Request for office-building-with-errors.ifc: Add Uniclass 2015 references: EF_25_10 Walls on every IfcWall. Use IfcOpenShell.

First a look at what the model holds.

```python
import ifcopenshell

model = ifcopenshell.open("office-building-with-errors.ifc")
print(model.schema)
print("classifications:", [c.Name for c in model.by_type("IfcClassification")])
for ifc_class in ("IfcDoor", "IfcRoof", "IfcStair", "IfcWall", "IfcWindow"):
    print(ifc_class, len(model.by_type(ifc_class)))
```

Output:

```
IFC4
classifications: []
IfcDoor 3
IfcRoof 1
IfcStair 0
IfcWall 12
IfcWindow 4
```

```python
import ifcopenshell
import ifcopenshell.api.classification

model = ifcopenshell.open("office-building-with-errors.ifc")

system = ifcopenshell.api.classification.add_classification(model, classification="Uniclass 2015")

codes = {
    "IfcWall": ("EF_25_10", "Walls"),
}
for ifc_class, (code, name) in codes.items():
    products = model.by_type(ifc_class)
    ifcopenshell.api.classification.add_reference(
        model, products=products, classification=system, identification=code, name=name
    )
    print(code, len(products))

model.write("office-building-with-errors-out.ifc")
```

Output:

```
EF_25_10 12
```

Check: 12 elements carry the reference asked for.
